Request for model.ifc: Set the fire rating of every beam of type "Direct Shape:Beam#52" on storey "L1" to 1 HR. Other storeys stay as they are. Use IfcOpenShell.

First a look at what the model holds.

```python
import ifcopenshell
import ifcopenshell.util.element

model = ifcopenshell.open("model.ifc")
print(model.schema)
storey = next(s for s in model.by_type("IfcBuildingStorey") if s.Name == "L1")
beams = [e for e in ifcopenshell.util.element.get_decomposition(storey) if e.is_a("IfcBeam")]
seen = {}
for e in beams:
    element_type = ifcopenshell.util.element.get_type(e)
    key = (element_type.Name if element_type != e and element_type else None, ifcopenshell.util.element.get_pset(e, "Pset_BeamCommon", "FireRating"))
    seen[key] = seen.get(key, 0) + 1
for (name, value), count in sorted(seen.items(), key=str):
    print(count, "x", name, "|", value)
```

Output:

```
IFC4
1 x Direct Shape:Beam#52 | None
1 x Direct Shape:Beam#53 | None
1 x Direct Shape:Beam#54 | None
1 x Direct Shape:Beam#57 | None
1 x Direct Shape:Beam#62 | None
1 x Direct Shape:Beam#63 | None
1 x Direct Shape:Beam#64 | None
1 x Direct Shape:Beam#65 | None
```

```python
import ifcopenshell
import ifcopenshell.api.pset
import ifcopenshell.util.element

model = ifcopenshell.open("model.ifc")

storey = next(s for s in model.by_type("IfcBuildingStorey") if s.Name == "L1")
beams = [e for e in ifcopenshell.util.element.get_decomposition(storey) if e.is_a("IfcBeam")]

count = 0
for e in beams:
    element_type = ifcopenshell.util.element.get_type(e)
    if element_type in (None, e) or element_type.Name != "Direct Shape:Beam#52":
        continue
    # add_pset returns the element's existing set when there is one.
    pset = ifcopenshell.api.pset.add_pset(model, product=e, name="Pset_BeamCommon")
    ifcopenshell.api.pset.edit_pset(model, pset=pset, properties={"FireRating": "1 HR"})
    count += 1

print(count, "beams updated")

model.write("model-out.ifc")
```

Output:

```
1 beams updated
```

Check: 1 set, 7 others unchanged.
